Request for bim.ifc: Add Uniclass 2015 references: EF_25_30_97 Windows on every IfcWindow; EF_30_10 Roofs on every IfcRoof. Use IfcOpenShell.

First a look at what the model holds.

```python
import ifcopenshell

model = ifcopenshell.open("bim.ifc")
print(model.schema)
print("classifications:", [c.Name for c in model.by_type("IfcClassification")])
for ifc_class in ("IfcDoor", "IfcRoof", "IfcStair", "IfcWall", "IfcWindow"):
    print(ifc_class, len(model.by_type(ifc_class)))
```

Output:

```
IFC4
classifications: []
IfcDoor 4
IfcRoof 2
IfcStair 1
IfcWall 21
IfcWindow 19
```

```python
import ifcopenshell
import ifcopenshell.api.classification

model = ifcopenshell.open("bim.ifc")

system = ifcopenshell.api.classification.add_classification(model, classification="Uniclass 2015")

codes = {
    "IfcWindow": ("EF_25_30_97", "Windows"),
    "IfcRoof": ("EF_30_10", "Roofs"),
}
for ifc_class, (code, name) in codes.items():
    products = model.by_type(ifc_class)
    ifcopenshell.api.classification.add_reference(
        model, products=products, classification=system, identification=code, name=name
    )
    print(code, len(products))

model.write("bim_rev.ifc")
```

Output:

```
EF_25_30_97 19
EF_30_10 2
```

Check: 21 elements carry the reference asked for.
